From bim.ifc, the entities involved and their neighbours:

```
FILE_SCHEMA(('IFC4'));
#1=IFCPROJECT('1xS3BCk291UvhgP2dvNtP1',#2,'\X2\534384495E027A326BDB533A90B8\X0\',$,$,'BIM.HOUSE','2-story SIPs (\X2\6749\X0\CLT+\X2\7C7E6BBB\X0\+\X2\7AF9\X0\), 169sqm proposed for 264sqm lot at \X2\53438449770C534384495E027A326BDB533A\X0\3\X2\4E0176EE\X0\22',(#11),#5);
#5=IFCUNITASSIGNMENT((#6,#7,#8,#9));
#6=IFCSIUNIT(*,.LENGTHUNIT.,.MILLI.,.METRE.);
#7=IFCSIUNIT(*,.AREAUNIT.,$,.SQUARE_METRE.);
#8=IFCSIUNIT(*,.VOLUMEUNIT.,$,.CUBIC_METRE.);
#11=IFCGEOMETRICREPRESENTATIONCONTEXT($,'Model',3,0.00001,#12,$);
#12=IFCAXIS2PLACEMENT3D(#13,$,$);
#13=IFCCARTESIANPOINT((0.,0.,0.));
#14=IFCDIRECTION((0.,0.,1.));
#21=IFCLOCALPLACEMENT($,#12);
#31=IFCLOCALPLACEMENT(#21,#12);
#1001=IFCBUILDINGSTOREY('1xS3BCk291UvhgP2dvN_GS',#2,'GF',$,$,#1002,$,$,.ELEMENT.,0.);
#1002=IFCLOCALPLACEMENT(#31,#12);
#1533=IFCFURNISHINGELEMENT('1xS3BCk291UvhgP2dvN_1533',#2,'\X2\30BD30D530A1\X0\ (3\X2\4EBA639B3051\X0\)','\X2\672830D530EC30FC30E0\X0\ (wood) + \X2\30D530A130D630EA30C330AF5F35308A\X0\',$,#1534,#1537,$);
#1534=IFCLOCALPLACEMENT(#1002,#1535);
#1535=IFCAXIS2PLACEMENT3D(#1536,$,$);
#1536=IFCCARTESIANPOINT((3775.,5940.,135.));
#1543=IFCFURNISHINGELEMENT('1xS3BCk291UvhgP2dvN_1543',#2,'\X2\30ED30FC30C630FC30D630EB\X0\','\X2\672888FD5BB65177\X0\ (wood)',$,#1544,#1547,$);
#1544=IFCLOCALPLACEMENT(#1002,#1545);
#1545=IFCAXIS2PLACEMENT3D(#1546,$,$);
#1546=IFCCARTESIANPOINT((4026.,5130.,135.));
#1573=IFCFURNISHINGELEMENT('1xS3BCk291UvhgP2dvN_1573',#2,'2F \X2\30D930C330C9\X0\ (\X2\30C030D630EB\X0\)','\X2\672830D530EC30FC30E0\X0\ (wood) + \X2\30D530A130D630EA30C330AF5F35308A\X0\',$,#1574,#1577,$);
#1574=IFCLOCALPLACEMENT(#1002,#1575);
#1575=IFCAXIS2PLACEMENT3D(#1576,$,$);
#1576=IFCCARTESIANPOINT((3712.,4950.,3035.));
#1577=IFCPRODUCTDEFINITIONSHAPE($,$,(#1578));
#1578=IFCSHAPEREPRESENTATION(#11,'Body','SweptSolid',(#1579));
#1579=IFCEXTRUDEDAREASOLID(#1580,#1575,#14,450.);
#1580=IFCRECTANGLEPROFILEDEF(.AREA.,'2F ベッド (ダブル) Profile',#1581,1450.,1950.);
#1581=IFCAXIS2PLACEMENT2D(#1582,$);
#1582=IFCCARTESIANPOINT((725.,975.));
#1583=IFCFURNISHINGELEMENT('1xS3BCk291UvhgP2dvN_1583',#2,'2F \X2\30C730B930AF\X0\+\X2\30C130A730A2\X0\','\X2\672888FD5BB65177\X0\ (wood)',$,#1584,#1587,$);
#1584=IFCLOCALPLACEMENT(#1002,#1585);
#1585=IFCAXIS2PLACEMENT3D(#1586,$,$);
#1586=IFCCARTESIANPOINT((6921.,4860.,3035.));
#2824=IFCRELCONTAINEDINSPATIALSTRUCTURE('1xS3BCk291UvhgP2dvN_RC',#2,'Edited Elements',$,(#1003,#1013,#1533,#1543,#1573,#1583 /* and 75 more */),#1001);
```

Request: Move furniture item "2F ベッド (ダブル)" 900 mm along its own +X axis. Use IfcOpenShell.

```python
import ifcopenshell
import ifcopenshell.api.geometry
import ifcopenshell.util.placement
import ifcopenshell.util.unit

model = ifcopenshell.open("bim.ifc")
unit_scale = ifcopenshell.util.unit.calculate_unit_scale(model)

item = model.by_guid("1xS3BCk291UvhgP2dvN_1573")
matrix = ifcopenshell.util.placement.get_local_placement(item.ObjectPlacement)
matrix[:3, 3] += matrix[:3, 0] * 0.9 / unit_scale
ifcopenshell.api.geometry.edit_object_placement(model, product=item, matrix=matrix, is_si=False)

print(ifcopenshell.util.placement.get_local_placement(item.ObjectPlacement).round(3) + 0.0)

model.write("bim_rev.ifc")
```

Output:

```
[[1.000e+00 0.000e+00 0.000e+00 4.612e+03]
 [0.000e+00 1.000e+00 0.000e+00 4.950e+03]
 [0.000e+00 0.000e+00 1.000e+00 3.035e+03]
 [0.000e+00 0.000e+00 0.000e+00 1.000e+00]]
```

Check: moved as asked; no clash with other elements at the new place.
